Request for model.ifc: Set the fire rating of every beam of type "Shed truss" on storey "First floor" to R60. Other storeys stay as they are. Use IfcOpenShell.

First a look at what the model holds.

```python
import ifcopenshell
import ifcopenshell.util.element

model = ifcopenshell.open("model.ifc")
print(model.schema)
storey = next(s for s in model.by_type("IfcBuildingStorey") if s.Name == "First floor")
beams = [e for e in ifcopenshell.util.element.get_decomposition(storey) if e.is_a("IfcBeam")]
seen = {}
for e in beams:
    element_type = ifcopenshell.util.element.get_type(e)
    key = (element_type.Name if element_type != e and element_type else None, ifcopenshell.util.element.get_pset(e, "Pset_BeamCommon", "FireRating"))
    seen[key] = seen.get(key, 0) + 1
for (name, value), count in sorted(seen.items(), key=str):
    print(count, "x", name, "|", value)
```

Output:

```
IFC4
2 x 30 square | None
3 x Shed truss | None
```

```python
import ifcopenshell
import ifcopenshell.api.pset
import ifcopenshell.util.element

model = ifcopenshell.open("model.ifc")

storey = next(s for s in model.by_type("IfcBuildingStorey") if s.Name == "First floor")
beams = [e for e in ifcopenshell.util.element.get_decomposition(storey) if e.is_a("IfcBeam")]

count = 0
for e in beams:
    element_type = ifcopenshell.util.element.get_type(e)
    if element_type in (None, e) or element_type.Name != "Shed truss":
        continue
    # add_pset returns the element's existing set when there is one.
    pset = ifcopenshell.api.pset.add_pset(model, product=e, name="Pset_BeamCommon")
    ifcopenshell.api.pset.edit_pset(model, pset=pset, properties={"FireRating": "R60"})
    count += 1

print(count, "beams updated")

model.write("model_rev.ifc")
```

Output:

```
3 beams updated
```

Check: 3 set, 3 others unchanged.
